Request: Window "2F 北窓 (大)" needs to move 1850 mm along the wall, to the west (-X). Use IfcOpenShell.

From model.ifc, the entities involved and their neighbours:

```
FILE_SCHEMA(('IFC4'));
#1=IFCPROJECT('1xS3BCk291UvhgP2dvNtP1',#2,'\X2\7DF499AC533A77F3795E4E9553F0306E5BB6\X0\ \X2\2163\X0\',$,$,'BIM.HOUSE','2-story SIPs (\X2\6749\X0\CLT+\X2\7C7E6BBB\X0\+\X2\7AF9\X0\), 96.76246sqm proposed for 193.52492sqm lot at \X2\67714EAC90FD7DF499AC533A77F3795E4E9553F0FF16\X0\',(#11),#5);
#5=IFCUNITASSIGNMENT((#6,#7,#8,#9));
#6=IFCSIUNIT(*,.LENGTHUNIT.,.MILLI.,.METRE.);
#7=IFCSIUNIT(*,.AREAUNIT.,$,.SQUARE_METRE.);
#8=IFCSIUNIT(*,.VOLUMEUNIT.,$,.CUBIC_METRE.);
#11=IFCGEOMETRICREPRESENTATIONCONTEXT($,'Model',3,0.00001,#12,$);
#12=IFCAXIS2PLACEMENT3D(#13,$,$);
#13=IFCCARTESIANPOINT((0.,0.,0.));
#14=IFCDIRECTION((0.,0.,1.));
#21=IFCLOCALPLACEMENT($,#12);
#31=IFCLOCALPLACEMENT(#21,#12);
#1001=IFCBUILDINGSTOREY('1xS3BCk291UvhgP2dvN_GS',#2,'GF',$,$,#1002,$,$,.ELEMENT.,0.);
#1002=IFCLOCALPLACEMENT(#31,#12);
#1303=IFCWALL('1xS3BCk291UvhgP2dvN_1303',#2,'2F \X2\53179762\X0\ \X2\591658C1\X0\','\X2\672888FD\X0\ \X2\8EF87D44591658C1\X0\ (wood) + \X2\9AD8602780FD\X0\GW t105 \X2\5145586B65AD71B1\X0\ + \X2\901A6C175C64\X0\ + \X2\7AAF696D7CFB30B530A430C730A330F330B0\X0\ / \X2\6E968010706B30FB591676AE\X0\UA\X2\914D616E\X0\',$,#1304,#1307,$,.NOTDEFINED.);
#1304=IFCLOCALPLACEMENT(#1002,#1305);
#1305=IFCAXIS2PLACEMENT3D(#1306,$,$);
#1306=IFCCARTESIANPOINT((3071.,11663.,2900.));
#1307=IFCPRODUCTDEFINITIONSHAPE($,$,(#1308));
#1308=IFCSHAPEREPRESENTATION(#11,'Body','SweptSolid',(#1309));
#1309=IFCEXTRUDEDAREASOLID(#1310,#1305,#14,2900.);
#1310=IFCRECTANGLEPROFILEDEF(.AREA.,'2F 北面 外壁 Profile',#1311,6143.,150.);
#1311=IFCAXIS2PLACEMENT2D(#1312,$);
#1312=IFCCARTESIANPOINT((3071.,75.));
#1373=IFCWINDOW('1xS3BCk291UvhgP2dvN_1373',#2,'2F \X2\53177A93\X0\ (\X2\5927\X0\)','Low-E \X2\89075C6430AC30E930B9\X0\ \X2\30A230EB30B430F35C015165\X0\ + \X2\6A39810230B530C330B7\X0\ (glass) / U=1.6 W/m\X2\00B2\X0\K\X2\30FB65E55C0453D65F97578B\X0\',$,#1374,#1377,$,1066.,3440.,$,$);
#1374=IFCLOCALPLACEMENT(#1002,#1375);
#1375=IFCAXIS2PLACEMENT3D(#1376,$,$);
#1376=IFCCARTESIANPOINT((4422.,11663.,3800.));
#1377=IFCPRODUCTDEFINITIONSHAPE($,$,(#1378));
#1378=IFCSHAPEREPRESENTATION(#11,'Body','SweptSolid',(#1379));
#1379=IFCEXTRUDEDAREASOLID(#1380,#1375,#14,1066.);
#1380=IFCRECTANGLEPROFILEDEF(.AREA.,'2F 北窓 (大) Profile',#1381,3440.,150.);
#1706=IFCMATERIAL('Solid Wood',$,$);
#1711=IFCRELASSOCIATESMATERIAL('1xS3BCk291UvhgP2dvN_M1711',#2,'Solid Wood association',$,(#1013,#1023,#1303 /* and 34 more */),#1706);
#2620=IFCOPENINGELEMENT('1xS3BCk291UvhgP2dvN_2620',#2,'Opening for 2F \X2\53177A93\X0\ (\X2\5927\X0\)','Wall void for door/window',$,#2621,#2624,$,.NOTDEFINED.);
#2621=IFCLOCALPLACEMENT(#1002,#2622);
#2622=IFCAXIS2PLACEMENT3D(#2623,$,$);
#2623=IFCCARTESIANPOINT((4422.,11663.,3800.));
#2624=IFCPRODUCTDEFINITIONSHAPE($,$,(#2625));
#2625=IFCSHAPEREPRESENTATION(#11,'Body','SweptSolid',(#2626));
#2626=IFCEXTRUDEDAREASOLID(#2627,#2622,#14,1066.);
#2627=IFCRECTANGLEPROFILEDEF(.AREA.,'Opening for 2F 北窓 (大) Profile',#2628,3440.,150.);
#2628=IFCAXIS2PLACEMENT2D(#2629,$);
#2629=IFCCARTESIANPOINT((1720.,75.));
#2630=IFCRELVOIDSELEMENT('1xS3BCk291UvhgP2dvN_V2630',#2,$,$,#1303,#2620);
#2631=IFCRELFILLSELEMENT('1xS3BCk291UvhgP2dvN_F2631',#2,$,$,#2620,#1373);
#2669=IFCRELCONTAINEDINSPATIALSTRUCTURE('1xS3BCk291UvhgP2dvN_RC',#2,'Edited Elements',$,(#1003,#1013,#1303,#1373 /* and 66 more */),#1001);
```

```python
import ifcopenshell
import ifcopenshell.api.geometry
import ifcopenshell.util.placement

model = ifcopenshell.open("model.ifc")

window = model.by_guid("1xS3BCk291UvhgP2dvN_1373")
opening = window.FillsVoids[0].RelatingOpeningElement
wall = opening.VoidsElements[0].RelatingBuildingElement

wall_matrix = ifcopenshell.util.placement.get_local_placement(wall.ObjectPlacement)
shift = wall_matrix[:3, 0] * -1850.0
before = ifcopenshell.util.placement.get_local_placement(window.ObjectPlacement)[:3, 3].copy()

# The window is not placed relative to its opening, so move both.
for product in (opening, window):
    matrix = ifcopenshell.util.placement.get_local_placement(product.ObjectPlacement)
    matrix[:3, 3] += shift
    ifcopenshell.api.geometry.edit_object_placement(model, product=product, matrix=matrix, is_si=False)

after = ifcopenshell.util.placement.get_local_placement(window.ObjectPlacement)[:3, 3]
print("window moved by", (after - before).round(3) + 0.0)

model.write("model_updated.ifc")
```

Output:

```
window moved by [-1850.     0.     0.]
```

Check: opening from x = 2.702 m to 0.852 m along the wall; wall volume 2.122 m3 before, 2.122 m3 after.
